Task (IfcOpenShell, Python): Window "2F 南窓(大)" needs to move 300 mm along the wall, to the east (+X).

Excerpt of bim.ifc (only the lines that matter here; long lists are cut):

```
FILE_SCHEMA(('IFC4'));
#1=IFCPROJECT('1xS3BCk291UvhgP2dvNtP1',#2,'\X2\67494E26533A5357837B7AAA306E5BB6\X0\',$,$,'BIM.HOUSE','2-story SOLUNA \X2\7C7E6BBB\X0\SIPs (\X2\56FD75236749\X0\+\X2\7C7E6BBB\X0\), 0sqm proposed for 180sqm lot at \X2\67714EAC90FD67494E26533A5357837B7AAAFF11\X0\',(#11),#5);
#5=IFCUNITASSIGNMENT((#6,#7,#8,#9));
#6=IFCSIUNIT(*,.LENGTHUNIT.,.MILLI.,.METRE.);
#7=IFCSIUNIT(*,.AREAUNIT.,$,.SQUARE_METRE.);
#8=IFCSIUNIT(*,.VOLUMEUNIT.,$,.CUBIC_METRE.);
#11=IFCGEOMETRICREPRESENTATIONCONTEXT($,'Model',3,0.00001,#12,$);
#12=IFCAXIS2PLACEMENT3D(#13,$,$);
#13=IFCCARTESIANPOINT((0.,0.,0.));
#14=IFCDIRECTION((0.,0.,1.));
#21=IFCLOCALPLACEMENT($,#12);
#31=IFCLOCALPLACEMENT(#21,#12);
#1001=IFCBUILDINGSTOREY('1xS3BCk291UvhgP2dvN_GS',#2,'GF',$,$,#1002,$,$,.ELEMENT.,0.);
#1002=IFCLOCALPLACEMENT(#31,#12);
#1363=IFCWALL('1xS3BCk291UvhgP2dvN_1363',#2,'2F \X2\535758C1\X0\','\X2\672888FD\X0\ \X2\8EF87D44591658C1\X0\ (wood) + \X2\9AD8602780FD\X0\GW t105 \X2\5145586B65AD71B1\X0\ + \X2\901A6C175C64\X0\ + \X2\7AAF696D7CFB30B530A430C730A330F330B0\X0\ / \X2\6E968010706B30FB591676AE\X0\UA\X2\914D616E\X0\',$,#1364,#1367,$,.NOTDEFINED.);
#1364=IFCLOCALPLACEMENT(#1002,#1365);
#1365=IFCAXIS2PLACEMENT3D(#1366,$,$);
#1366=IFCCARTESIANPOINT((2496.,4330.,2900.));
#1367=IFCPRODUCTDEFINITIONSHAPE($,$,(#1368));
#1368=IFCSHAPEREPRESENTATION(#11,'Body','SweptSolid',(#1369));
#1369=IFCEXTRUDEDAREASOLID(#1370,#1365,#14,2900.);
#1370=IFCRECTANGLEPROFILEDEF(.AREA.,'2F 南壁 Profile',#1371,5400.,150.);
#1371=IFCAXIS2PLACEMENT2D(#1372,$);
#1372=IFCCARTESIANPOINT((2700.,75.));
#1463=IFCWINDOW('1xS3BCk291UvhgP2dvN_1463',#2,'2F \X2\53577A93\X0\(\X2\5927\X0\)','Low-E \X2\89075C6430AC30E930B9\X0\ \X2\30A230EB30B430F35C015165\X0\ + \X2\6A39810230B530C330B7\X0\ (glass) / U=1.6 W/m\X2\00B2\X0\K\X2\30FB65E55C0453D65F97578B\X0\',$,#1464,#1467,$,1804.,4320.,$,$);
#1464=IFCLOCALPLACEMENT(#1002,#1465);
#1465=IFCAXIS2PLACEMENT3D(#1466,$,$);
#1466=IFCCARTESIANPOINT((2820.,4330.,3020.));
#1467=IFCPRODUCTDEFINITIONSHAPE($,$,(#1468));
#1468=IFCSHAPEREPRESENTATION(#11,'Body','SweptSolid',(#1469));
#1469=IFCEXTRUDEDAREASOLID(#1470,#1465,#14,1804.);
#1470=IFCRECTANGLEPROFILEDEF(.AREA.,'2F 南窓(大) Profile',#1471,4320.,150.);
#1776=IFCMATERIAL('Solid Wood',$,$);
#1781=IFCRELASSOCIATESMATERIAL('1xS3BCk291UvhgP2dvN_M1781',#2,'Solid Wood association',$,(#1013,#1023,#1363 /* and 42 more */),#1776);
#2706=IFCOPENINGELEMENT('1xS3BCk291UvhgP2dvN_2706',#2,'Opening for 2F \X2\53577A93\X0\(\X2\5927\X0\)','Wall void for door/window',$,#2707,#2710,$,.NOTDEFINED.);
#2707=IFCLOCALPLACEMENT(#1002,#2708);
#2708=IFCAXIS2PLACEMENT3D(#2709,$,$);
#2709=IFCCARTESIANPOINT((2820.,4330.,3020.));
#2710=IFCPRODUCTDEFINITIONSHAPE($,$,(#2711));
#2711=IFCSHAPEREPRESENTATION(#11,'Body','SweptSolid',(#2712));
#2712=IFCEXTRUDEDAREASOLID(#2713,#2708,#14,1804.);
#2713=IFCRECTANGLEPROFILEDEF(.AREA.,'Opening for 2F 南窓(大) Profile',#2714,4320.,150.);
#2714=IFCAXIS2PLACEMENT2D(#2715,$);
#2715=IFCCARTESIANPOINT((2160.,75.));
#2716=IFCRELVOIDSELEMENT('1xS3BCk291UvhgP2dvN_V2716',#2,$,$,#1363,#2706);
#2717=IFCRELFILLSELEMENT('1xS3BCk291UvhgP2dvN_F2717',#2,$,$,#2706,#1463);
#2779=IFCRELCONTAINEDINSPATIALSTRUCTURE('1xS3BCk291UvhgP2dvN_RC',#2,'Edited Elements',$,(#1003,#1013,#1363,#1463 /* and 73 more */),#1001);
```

```python
import ifcopenshell
import ifcopenshell.api.geometry
import ifcopenshell.util.placement
import ifcopenshell.util.unit

model = ifcopenshell.open("bim.ifc")
unit_scale = ifcopenshell.util.unit.calculate_unit_scale(model)

window = model.by_id(1463)
opening = window.FillsVoids[0].RelatingOpeningElement
wall = opening.VoidsElements[0].RelatingBuildingElement

wall_matrix = ifcopenshell.util.placement.get_local_placement(wall.ObjectPlacement)
shift = wall_matrix[:3, 0] * 0.3 / unit_scale
before = ifcopenshell.util.placement.get_local_placement(window.ObjectPlacement)[:3, 3].copy()

# The window is not placed relative to its opening, so move both.
for product in (opening, window):
    matrix = ifcopenshell.util.placement.get_local_placement(product.ObjectPlacement)
    matrix[:3, 3] += shift
    ifcopenshell.api.geometry.edit_object_placement(model, product=product, matrix=matrix, is_si=False)

after = ifcopenshell.util.placement.get_local_placement(window.ObjectPlacement)[:3, 3]
print("window moved by", (after - before).round(3) + 0.0)

model.write("bim-out.ifc")
```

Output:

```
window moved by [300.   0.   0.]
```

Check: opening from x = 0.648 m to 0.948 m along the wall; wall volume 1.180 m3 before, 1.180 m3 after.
